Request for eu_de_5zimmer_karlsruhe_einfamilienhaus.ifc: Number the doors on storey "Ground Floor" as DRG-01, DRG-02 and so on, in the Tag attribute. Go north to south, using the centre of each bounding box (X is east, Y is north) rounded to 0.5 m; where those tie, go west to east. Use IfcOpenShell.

First a look at what the model holds.

```python
import ifcopenshell
import ifcopenshell.util.element
import ifcopenshell.util.placement

model = ifcopenshell.open("eu_de_5zimmer_karlsruhe_einfamilienhaus.ifc")
print(model.schema)
storey = next(s for s in model.by_type("IfcBuildingStorey") if s.Name == "Ground Floor")
doors = [e for e in ifcopenshell.util.element.get_decomposition(storey) if e.is_a("IfcDoor")]
for e in sorted(doors, key=lambda e: e.id()):
    origin = ifcopenshell.util.placement.get_local_placement(e.ObjectPlacement)[:3, 3]
    print(e.id(), e.Tag, e.Name, origin.round(2) + 0.0, sep=" | ")
```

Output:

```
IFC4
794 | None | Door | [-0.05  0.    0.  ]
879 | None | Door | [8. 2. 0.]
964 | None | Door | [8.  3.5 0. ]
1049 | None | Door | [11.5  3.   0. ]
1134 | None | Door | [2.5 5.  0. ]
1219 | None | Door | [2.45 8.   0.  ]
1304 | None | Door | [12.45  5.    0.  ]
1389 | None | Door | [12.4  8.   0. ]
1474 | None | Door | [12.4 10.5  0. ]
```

```python
import ifcopenshell
import ifcopenshell.geom
import ifcopenshell.util.element
import ifcopenshell.util.shape

model = ifcopenshell.open("eu_de_5zimmer_karlsruhe_einfamilienhaus.ifc")
settings = ifcopenshell.geom.settings()
settings.set("use-world-coords", True)


def centre(element):
    shape = ifcopenshell.geom.create_shape(settings, element)
    return ifcopenshell.util.shape.get_bbox_centroid(shape.geometry)


storey = next(s for s in model.by_type("IfcBuildingStorey") if s.Name == "Ground Floor")
doors = [e for e in ifcopenshell.util.element.get_decomposition(storey) if e.is_a("IfcDoor")]

# Insertion points can sit at a corner or the storey origin, so sort by the geometry (in metres).
centres = {e: centre(e) for e in doors}
doors.sort(key=lambda e: (-round(centres[e][1] / 0.5), centres[e][0]))

for i, e in enumerate(doors, start=1):
    number = f"DRG-{i:02d}"
    e.Tag = number
    print(e.id(), number)

model.write("eu_de_5zimmer_karlsruhe_einfamilienhaus_v2.ifc")
```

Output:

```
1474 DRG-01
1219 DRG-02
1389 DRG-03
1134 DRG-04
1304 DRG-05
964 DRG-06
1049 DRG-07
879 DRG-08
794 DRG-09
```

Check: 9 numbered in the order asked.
